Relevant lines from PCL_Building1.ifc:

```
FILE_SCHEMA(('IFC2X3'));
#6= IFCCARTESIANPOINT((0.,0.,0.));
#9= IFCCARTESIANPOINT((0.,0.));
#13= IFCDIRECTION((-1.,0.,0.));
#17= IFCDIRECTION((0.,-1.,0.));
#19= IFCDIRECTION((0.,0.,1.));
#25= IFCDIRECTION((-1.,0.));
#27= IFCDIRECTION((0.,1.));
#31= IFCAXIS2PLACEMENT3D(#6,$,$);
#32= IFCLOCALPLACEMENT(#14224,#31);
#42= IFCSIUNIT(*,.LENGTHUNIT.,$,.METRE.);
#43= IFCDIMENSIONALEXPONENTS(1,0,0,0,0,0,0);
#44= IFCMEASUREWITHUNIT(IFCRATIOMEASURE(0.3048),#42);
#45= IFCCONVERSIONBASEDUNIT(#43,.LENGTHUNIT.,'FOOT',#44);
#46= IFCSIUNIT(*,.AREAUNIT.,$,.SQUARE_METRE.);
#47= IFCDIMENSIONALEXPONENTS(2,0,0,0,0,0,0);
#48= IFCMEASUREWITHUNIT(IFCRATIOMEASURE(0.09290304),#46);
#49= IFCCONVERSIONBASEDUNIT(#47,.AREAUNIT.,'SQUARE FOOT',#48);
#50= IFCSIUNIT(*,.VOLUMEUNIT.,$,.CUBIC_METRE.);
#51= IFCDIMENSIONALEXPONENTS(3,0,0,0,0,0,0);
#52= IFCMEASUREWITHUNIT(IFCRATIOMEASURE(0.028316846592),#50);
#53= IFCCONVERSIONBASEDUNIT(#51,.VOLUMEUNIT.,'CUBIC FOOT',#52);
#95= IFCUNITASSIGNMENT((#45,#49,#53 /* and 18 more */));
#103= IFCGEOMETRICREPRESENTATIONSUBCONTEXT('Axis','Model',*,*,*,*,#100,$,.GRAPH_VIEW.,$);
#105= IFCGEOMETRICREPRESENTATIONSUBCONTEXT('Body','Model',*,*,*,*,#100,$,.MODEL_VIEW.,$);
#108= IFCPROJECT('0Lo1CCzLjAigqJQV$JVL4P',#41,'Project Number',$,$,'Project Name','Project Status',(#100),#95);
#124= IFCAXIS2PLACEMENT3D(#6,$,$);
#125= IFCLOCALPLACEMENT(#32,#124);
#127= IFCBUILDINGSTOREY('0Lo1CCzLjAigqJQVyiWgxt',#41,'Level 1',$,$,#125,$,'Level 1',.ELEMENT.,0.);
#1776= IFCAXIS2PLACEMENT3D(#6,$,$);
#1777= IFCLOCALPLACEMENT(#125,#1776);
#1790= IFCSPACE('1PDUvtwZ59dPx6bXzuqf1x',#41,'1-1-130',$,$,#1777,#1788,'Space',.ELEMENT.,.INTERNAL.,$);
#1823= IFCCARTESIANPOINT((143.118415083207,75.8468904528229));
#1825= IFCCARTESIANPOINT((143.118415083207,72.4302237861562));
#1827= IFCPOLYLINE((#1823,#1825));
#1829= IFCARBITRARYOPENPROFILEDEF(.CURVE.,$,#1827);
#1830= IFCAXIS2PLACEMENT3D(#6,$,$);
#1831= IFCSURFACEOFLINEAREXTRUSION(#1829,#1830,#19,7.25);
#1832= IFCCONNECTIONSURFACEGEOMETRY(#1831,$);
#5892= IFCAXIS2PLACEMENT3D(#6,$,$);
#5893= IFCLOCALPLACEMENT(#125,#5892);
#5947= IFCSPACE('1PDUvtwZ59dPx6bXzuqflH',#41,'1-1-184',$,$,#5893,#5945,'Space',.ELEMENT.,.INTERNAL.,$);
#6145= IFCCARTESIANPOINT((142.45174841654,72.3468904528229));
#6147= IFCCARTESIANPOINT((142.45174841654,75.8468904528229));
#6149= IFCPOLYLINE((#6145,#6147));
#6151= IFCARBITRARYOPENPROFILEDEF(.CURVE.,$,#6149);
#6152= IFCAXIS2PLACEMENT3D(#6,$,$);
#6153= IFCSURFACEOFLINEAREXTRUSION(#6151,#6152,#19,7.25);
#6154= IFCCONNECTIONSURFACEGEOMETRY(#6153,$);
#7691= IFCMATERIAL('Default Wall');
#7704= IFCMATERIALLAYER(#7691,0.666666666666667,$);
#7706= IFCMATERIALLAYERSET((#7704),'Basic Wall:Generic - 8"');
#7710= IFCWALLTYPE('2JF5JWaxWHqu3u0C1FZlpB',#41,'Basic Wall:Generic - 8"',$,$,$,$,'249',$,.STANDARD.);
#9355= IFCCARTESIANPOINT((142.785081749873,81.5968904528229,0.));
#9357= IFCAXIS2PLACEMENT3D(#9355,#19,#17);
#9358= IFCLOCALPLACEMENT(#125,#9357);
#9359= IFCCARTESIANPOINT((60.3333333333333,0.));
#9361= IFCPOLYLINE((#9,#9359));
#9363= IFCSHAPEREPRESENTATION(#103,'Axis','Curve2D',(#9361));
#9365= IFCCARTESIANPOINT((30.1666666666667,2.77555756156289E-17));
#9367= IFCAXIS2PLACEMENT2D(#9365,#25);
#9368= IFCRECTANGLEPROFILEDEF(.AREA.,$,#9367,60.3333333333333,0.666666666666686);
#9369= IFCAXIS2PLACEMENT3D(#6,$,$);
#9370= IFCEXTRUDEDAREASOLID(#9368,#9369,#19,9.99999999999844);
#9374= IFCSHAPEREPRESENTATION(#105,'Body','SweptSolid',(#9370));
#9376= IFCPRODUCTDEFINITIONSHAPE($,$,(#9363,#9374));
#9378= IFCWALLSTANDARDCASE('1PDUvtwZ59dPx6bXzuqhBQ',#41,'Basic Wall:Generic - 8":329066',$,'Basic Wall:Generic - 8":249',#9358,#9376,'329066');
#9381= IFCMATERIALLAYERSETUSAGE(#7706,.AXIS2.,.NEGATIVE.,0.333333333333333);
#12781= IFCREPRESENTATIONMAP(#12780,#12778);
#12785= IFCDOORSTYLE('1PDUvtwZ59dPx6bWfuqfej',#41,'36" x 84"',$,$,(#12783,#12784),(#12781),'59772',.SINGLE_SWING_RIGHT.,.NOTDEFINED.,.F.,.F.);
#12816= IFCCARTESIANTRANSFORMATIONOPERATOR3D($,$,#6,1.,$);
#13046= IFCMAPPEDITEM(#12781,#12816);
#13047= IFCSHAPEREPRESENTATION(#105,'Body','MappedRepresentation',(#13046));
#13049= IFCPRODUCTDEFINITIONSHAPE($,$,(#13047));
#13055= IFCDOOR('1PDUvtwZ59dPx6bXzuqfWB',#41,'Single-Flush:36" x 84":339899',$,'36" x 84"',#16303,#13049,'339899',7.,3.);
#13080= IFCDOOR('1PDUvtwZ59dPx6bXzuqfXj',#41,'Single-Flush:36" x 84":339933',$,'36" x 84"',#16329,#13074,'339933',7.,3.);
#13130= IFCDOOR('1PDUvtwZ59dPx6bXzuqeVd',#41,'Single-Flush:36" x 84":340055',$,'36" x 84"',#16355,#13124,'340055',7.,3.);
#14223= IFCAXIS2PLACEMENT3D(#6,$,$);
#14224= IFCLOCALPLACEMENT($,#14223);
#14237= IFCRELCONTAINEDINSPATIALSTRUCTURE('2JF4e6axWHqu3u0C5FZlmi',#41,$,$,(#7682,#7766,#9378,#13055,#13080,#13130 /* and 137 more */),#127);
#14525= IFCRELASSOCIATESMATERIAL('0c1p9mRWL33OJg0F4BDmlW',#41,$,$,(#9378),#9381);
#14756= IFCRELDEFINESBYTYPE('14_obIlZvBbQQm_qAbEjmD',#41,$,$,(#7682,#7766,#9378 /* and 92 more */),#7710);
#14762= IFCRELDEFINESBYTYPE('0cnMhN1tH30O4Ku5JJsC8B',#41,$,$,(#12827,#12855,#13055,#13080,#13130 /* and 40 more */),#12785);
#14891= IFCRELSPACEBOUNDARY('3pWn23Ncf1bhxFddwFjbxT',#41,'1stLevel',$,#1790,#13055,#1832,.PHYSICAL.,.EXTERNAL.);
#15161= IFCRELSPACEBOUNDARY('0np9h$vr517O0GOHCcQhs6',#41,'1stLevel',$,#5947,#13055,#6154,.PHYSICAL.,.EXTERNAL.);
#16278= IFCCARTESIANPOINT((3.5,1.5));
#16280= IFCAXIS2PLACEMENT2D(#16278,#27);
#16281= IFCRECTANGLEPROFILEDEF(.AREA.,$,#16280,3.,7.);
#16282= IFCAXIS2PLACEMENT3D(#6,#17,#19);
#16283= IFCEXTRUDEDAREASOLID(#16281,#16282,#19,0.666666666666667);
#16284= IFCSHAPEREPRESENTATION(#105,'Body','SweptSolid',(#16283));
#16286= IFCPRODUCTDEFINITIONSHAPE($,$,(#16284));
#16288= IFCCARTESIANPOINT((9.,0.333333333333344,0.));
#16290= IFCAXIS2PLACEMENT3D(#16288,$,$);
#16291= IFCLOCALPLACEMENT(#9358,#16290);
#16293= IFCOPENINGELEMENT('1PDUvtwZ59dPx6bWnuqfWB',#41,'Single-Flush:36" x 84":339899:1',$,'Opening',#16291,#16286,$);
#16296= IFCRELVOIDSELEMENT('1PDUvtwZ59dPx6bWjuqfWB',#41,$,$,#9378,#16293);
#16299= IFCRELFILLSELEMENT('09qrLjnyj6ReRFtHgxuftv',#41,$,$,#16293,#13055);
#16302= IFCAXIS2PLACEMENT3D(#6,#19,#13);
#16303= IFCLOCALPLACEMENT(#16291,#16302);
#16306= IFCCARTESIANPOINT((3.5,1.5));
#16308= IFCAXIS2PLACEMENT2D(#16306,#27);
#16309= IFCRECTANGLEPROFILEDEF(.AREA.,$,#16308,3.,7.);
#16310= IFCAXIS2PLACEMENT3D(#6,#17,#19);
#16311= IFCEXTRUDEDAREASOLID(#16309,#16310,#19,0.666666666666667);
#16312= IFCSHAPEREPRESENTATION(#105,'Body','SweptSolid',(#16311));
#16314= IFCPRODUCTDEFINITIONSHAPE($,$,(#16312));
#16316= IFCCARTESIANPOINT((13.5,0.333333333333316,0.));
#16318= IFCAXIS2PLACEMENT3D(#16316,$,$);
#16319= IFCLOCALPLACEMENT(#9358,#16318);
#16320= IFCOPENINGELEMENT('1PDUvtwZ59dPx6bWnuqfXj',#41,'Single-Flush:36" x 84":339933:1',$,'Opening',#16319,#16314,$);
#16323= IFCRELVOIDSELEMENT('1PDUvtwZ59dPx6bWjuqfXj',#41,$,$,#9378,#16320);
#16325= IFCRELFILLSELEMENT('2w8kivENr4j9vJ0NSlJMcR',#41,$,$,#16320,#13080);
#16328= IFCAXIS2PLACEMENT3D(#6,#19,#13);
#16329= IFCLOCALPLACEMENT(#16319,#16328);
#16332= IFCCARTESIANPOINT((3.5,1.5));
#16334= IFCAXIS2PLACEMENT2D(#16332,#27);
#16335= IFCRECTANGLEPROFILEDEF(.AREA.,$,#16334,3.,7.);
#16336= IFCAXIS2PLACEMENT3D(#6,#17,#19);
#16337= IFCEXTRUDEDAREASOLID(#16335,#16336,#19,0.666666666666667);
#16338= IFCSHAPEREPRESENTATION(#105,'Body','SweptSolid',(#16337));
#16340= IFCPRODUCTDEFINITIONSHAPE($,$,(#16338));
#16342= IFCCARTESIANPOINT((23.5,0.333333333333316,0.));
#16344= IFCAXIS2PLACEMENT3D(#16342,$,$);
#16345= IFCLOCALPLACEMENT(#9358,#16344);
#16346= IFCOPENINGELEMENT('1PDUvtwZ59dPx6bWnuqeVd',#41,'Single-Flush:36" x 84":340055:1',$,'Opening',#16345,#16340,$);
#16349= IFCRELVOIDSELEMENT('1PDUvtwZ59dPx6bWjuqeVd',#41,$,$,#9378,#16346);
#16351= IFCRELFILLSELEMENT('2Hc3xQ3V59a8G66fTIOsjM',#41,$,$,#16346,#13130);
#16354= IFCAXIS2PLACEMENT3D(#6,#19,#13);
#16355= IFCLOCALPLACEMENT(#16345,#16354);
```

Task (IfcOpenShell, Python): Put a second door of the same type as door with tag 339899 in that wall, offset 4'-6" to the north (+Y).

```python
import numpy as np
import ifcopenshell
import ifcopenshell.api.feature
import ifcopenshell.api.geometry
import ifcopenshell.api.root
import ifcopenshell.geom
import ifcopenshell.util.element
import ifcopenshell.util.placement
import ifcopenshell.util.shape
import ifcopenshell.util.unit

model = ifcopenshell.open("PCL_Building1.ifc")
unit_scale = ifcopenshell.util.unit.calculate_unit_scale(model)
settings = ifcopenshell.geom.settings()


def volume(element):
    """Net volume in cubic metres, openings subtracted."""
    shape = ifcopenshell.geom.create_shape(settings, element)
    return ifcopenshell.util.shape.get_volume(shape.geometry)


def reuse_history(source, copy):
    """copy_class also copies each property set's owner history, people and application; keep the originals."""
    for rel in copy.IsDefinedBy:
        if rel.is_a("IfcRelDefinesByProperties") and (history := rel.RelatingPropertyDefinition.OwnerHistory):
            rel.RelatingPropertyDefinition.OwnerHistory = source.OwnerHistory
            ifcopenshell.util.element.remove_deep2(model, history)


door = model.by_guid("1PDUvtwZ59dPx6bXzuqfWB")
opening = door.FillsVoids[0].RelatingOpeningElement
wall = opening.VoidsElements[0].RelatingBuildingElement
before = volume(wall)
shift = ifcopenshell.util.placement.get_local_placement(wall.ObjectPlacement)[:3, 0] * -54 * 0.0254 / unit_scale

# copy_class copies the void relationship, type, container and properties, but no geometry.
new_opening = ifcopenshell.api.root.copy_class(model, product=opening)
new_opening.Representation = ifcopenshell.util.element.copy_deep(
    model, opening.Representation, exclude=["IfcGeometricRepresentationContext", "IfcRepresentationMap"]
)
new_opening.Name = 'Single-Flush:36" x 84"'
new_door = ifcopenshell.api.root.copy_class(model, product=door)
new_door.Representation = ifcopenshell.util.element.copy_deep(
    model, door.Representation, exclude=["IfcGeometricRepresentationContext", "IfcRepresentationMap"]
)
new_door.Name = 'Single-Flush:36" x 84"'
new_door.Tag = None
reuse_history(door, new_door)
fills = ifcopenshell.api.feature.add_filling(model, opening=new_opening, element=new_door)
fills.OwnerHistory = new_door.OwnerHistory  # required in IFC2X3

for old, new in ((opening, new_opening), (door, new_door)):
    matrix = ifcopenshell.util.placement.get_local_placement(old.ObjectPlacement)
    matrix[:3, 3] += shift
    ifcopenshell.api.geometry.edit_object_placement(model, product=new, matrix=matrix, is_si=False)

# The copied space boundaries still share their surfaces with the original.
for rel in new_door.ProvidesBoundaries:
    if rel.ConnectionGeometry:
        rel.ConnectionGeometry = ifcopenshell.util.element.copy_deep(model, rel.ConnectionGeometry)

# Space boundary surfaces are stored in each space's coordinates; move them too.
for rel in new_door.ProvidesBoundaries:
    if not rel.ConnectionGeometry:
        continue
    surface = rel.ConnectionGeometry.SurfaceOnRelatingElement
    space_matrix = ifcopenshell.util.placement.get_local_placement(rel.RelatingSpace.ObjectPlacement)
    point = np.array(surface.Position.Location.Coordinates) + space_matrix[:3, :3].T @ shift
    surface.Position = model.createIfcAxis2Placement3D(
        model.createIfcCartesianPoint(point.tolist()), surface.Position.Axis, surface.Position.RefDirection
    )

after = volume(wall)

print(f"wall volume {before:.3f} -> {after:.3f} m3")

model.write("PCL_Building1_edited.ifc")
```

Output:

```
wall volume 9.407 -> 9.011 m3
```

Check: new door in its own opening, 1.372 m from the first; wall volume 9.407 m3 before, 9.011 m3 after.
